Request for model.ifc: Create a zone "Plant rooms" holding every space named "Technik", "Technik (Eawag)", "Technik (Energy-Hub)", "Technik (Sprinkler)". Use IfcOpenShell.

First a look at what the model holds.

```python
import ifcopenshell

model = ifcopenshell.open("model.ifc")
print(model.schema)
seen = {}
for space in model.by_type("IfcSpace"):
    seen[space.LongName] = seen.get(space.LongName, 0) + 1
for name, count in sorted(seen.items(), key=str):
    print(count, "x", name)
print("zones:", [z.Name for z in model.by_type("IfcZone")][:20])
```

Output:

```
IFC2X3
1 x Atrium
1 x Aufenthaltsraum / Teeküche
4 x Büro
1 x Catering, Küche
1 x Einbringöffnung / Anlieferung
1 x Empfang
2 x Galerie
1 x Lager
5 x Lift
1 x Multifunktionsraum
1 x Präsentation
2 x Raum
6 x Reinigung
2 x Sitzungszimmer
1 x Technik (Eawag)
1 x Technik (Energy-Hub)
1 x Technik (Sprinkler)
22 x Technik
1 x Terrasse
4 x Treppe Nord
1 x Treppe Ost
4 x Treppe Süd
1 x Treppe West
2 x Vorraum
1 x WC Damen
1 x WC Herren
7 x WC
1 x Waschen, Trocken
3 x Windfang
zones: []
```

```python
import ifcopenshell
import ifcopenshell.api.group
import ifcopenshell.api.root

model = ifcopenshell.open("model.ifc")

names = {"Technik", "Technik (Eawag)", "Technik (Energy-Hub)", "Technik (Sprinkler)"}
spaces = [s for s in model.by_type("IfcSpace") if s.LongName in names]

zone = ifcopenshell.api.root.create_entity(model, ifc_class="IfcZone", name="Plant rooms")
ifcopenshell.api.group.assign_group(model, products=spaces, group=zone)
print(len(spaces), "spaces in", zone.Name)

model.write("model_v2.ifc")
```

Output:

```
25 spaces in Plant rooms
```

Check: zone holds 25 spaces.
